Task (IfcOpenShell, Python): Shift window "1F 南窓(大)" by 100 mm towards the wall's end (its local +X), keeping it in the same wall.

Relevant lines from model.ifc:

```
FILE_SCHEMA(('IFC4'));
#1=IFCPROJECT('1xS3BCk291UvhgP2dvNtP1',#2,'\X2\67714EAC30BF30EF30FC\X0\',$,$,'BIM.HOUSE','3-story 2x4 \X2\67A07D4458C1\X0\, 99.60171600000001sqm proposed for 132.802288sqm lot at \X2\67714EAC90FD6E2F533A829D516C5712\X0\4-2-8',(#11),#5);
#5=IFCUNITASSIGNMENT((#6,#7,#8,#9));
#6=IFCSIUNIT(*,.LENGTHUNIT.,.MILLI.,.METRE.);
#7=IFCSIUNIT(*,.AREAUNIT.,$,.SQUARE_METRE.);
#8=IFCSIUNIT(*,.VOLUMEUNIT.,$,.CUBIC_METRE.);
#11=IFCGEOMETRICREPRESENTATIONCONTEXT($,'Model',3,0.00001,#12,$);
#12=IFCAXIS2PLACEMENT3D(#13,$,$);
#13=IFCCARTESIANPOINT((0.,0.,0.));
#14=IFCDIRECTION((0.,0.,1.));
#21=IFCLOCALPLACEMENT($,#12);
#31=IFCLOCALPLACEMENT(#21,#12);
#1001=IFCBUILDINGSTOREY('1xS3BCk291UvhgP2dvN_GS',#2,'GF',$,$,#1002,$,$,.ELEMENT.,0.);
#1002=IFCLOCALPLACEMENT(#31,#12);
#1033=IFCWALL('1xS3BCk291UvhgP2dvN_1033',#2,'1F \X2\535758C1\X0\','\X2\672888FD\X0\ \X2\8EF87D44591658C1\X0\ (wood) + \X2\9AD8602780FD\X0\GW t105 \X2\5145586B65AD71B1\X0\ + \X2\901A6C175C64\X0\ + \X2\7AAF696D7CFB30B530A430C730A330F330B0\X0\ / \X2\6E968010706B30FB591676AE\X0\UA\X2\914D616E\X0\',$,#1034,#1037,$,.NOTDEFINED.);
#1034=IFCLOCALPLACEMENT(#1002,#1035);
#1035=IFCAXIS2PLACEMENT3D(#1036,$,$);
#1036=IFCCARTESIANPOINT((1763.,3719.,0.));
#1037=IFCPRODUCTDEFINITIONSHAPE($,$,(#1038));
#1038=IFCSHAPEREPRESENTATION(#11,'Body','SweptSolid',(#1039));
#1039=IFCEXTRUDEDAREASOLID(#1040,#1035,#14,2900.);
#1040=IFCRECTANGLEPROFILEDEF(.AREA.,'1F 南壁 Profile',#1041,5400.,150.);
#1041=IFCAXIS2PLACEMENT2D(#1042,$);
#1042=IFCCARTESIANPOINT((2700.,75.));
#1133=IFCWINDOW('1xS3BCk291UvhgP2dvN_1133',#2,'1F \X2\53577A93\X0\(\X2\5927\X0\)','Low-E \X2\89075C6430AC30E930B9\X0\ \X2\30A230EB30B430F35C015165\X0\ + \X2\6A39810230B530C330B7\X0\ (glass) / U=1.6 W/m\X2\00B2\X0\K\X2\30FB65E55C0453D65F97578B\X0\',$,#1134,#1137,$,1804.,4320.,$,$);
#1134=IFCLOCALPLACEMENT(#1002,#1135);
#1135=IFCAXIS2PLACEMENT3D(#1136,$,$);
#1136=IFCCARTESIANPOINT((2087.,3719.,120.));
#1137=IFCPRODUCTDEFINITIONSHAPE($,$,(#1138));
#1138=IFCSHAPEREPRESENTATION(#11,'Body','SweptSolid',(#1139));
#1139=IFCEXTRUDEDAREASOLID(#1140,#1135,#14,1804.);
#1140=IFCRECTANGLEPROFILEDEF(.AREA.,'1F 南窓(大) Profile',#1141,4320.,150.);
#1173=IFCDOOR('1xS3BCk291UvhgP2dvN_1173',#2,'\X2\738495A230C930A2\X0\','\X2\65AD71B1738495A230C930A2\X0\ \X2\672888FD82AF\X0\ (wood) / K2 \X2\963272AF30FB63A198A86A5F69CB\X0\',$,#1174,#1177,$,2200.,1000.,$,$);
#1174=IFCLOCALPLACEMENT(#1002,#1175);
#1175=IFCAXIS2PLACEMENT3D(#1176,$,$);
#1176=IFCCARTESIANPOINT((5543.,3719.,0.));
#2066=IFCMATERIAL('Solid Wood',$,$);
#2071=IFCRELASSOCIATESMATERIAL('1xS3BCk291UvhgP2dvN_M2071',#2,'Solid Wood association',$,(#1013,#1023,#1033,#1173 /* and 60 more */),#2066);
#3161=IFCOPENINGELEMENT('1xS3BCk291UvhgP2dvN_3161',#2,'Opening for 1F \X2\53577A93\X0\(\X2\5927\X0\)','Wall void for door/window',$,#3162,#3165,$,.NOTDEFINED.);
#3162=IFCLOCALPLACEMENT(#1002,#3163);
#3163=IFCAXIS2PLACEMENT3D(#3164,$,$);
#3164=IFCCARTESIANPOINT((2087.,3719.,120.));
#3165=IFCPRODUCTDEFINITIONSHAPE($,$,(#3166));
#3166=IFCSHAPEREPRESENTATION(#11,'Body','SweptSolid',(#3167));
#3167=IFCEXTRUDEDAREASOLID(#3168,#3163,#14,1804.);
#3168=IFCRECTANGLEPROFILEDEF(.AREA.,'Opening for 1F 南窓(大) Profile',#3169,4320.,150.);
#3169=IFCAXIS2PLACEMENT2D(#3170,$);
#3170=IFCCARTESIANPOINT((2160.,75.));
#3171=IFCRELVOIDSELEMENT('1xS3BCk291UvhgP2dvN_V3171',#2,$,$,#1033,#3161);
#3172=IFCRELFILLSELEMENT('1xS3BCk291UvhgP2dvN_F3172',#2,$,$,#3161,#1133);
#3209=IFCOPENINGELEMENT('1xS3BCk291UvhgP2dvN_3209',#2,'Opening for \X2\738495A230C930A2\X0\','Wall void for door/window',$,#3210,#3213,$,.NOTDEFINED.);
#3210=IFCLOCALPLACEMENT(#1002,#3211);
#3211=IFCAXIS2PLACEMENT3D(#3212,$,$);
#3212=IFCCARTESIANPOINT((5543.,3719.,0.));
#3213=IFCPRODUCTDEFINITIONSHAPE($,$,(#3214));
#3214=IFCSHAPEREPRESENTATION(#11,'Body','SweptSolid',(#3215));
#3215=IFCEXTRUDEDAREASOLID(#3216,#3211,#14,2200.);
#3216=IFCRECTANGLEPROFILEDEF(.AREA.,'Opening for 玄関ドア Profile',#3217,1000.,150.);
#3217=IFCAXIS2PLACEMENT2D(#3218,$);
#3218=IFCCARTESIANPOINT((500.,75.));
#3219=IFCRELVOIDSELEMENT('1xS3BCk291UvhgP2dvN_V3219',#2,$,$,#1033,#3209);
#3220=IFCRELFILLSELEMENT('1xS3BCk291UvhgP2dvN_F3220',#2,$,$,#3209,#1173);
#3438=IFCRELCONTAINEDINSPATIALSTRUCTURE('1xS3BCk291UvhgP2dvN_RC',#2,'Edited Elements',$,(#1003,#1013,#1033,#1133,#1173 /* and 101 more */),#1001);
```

```python
import ifcopenshell
import ifcopenshell.api.geometry
import ifcopenshell.util.placement
import ifcopenshell.util.unit

model = ifcopenshell.open("model.ifc")
unit_scale = ifcopenshell.util.unit.calculate_unit_scale(model)

window = model.by_id(1133)
opening = window.FillsVoids[0].RelatingOpeningElement
wall = opening.VoidsElements[0].RelatingBuildingElement

wall_matrix = ifcopenshell.util.placement.get_local_placement(wall.ObjectPlacement)
shift = wall_matrix[:3, 0] * 0.1 / unit_scale
before = ifcopenshell.util.placement.get_local_placement(window.ObjectPlacement)[:3, 3].copy()

# The window is not placed relative to its opening, so move both.
for product in (opening, window):
    matrix = ifcopenshell.util.placement.get_local_placement(product.ObjectPlacement)
    matrix[:3, 3] += shift
    ifcopenshell.api.geometry.edit_object_placement(model, product=product, matrix=matrix, is_si=False)

after = ifcopenshell.util.placement.get_local_placement(window.ObjectPlacement)[:3, 3]
print("window moved by", (after - before).round(3) + 0.0)

model.write("model-out.ifc")
```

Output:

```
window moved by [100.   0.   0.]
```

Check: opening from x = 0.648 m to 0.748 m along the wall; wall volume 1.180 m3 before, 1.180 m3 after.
